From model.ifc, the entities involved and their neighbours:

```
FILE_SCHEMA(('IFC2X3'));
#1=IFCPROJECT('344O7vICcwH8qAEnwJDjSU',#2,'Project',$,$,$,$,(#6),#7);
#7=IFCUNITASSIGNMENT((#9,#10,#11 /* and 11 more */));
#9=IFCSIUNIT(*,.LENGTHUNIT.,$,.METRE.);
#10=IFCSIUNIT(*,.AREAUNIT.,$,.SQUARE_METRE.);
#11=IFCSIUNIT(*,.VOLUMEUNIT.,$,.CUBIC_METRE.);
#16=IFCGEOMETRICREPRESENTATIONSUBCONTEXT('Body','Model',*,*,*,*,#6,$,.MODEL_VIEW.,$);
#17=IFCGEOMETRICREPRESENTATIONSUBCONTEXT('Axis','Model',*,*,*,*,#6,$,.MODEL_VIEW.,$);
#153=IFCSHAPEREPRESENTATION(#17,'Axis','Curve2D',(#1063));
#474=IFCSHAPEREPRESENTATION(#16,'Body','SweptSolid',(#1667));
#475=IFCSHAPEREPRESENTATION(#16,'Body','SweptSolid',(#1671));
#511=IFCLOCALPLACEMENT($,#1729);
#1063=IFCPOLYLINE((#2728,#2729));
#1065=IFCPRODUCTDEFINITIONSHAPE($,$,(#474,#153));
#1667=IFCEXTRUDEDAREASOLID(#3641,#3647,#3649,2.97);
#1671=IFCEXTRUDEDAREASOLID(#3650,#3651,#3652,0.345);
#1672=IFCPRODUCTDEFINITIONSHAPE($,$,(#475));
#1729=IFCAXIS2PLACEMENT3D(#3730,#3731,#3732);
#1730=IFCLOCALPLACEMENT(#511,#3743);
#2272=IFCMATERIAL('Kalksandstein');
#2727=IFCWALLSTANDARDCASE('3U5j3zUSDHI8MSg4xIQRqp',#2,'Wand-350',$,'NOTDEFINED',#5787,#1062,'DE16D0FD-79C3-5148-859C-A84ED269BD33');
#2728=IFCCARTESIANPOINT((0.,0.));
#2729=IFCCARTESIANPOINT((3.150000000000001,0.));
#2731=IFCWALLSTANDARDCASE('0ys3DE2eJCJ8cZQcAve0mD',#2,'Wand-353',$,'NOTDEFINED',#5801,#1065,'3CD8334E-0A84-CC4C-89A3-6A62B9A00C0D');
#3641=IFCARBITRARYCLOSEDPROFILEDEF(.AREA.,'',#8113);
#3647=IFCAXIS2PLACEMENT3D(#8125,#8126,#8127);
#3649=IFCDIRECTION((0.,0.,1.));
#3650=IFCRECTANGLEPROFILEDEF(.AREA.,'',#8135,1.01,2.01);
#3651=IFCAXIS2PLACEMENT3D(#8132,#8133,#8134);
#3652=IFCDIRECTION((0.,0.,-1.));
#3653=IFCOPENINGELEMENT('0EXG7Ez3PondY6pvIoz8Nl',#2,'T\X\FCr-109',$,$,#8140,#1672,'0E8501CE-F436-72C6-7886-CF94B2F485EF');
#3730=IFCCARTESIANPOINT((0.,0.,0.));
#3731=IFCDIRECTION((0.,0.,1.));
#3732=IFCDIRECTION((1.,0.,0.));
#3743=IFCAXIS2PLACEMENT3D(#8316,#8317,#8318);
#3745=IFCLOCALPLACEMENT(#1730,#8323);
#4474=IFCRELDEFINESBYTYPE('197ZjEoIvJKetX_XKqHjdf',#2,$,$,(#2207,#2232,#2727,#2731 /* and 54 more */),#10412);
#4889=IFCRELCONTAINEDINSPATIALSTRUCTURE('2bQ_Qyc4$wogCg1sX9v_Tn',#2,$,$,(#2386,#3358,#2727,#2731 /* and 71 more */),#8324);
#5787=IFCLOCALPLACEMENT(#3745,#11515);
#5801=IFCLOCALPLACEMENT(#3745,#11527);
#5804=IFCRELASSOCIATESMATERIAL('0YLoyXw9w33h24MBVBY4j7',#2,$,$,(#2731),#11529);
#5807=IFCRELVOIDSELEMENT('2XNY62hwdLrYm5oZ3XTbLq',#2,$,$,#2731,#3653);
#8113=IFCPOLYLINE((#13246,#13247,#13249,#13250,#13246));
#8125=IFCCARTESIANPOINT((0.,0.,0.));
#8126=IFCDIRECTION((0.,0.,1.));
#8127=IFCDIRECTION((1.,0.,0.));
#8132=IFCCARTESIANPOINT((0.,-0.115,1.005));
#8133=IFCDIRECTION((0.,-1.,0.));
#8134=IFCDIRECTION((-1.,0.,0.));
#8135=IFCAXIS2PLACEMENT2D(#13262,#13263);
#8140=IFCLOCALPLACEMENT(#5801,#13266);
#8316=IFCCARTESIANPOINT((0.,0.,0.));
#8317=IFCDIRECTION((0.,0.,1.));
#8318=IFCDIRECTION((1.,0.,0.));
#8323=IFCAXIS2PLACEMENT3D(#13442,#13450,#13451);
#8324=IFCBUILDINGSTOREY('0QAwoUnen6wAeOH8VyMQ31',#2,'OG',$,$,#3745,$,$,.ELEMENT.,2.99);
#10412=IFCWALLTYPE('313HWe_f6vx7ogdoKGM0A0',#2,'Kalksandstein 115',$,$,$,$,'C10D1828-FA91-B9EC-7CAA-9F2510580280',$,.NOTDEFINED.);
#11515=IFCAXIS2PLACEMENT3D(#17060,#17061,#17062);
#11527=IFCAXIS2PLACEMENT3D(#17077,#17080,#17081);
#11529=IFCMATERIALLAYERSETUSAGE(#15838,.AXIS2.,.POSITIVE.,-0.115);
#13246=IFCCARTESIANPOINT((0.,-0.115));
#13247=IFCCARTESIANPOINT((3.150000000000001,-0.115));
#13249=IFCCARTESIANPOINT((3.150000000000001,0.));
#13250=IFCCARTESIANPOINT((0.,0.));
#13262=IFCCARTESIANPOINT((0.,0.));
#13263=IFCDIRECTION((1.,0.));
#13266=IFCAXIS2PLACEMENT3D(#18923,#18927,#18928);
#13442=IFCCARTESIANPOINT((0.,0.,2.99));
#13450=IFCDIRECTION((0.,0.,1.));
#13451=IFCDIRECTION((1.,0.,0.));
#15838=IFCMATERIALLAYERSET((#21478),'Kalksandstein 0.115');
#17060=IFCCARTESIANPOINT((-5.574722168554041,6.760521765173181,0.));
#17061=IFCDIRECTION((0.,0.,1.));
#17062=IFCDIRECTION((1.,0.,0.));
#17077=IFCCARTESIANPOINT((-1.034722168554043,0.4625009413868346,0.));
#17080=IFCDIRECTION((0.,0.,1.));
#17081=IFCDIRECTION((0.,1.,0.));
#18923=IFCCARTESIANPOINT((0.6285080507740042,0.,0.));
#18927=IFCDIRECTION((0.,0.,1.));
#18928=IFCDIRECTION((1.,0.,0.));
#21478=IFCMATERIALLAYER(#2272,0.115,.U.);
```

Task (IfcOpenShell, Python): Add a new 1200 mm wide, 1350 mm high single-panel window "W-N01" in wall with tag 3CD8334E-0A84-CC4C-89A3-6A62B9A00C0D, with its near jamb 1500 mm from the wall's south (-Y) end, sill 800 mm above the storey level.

```python
import numpy as np
import ifcopenshell
import ifcopenshell.api.feature
import ifcopenshell.api.geometry
import ifcopenshell.api.root
import ifcopenshell.api.spatial
import ifcopenshell.api.type
import ifcopenshell.geom
import ifcopenshell.util.element
import ifcopenshell.util.placement
import ifcopenshell.util.representation
import ifcopenshell.util.shape
import ifcopenshell.util.unit

model = ifcopenshell.open("model.ifc")
unit_scale = ifcopenshell.util.unit.calculate_unit_scale(model)
settings = ifcopenshell.geom.settings()


def volume(element):
    """Net volume in cubic metres, openings subtracted."""
    shape = ifcopenshell.geom.create_shape(settings, element)
    return ifcopenshell.util.shape.get_volume(shape.geometry)


wall = model.by_guid("0ys3DE2eJCJ8cZQcAve0mD")
storey = ifcopenshell.util.element.get_container(wall, ifc_class="IfcBuildingStorey")
context = ifcopenshell.util.representation.get_context(model, "Model", "Body", "MODEL_VIEW")
before = volume(wall)

width, height, from_end, sill = 1.2, 1.35, 1.5, 0.8  # metres

# The wall runs along its own X axis, and the end named is its -X end.
wall_shape = ifcopenshell.geom.create_shape(settings, wall)
x, y, z = ifcopenshell.util.shape.get_vertices(wall_shape.geometry).T
start = x.min() + from_end
face, thickness = float(y.min()), float(y.max() - y.min())
wall_matrix = ifcopenshell.util.placement.get_local_placement(wall.ObjectPlacement)
level = ifcopenshell.util.placement.get_local_placement(storey.ObjectPlacement)[2, 3]


def in_wall(x, y):
    """Placement at x, y metres in the wall's axes, at sill height."""
    matrix = wall_matrix.copy()
    matrix[:, 3] = wall_matrix @ np.array([x / unit_scale, y / unit_scale, 0.0, 1.0])
    matrix[2, 3] = level + sill / unit_scale
    return matrix


# Opening: a box that overshoots both wall faces by 50 mm.
opening = ifcopenshell.api.root.create_entity(model, ifc_class="IfcOpeningElement")
box = ifcopenshell.api.geometry.add_wall_representation(
    model, context=context, length=width, height=height, thickness=thickness + 0.1
)
ifcopenshell.api.geometry.assign_representation(model, product=opening, representation=box)
ifcopenshell.api.geometry.edit_object_placement(model, product=opening, matrix=in_wall(start, face - 0.05), is_si=False)
ifcopenshell.api.feature.add_feature(model, feature=opening, element=wall)

window = ifcopenshell.api.root.create_entity(model, ifc_class="IfcWindow", name="W-N01")
window.OverallWidth, window.OverallHeight = width / unit_scale, height / unit_scale
body = ifcopenshell.api.geometry.add_window_representation(
    model,
    context=context,
    overall_width=window.OverallWidth,
    overall_height=window.OverallHeight,
    partition_type="SINGLE_PANEL",
)
ifcopenshell.api.geometry.assign_representation(model, product=window, representation=body)
ifcopenshell.api.spatial.assign_container(model, products=[window], relating_structure=storey)
fills = ifcopenshell.api.feature.add_filling(model, opening=opening, element=window)
fills.OwnerHistory = window.OwnerHistory  # required in IFC2X3

# IFC2X3 keeps the operation on the window style.
style = ifcopenshell.api.root.create_entity(model, ifc_class="IfcWindowStyle", name="W-N01")
style.OperationType, style.ConstructionType = "SINGLE_PANEL", "NOTDEFINED"
style.ParameterTakesPrecedence = style.Sizeable = False
ifcopenshell.api.type.assign_type(model, related_objects=[window], relating_type=style)

# Centre the window in the wall's thickness.
ifcopenshell.api.geometry.edit_object_placement(model, product=window, matrix=in_wall(start, face), is_si=False)
window_shape = ifcopenshell.geom.create_shape(settings, window)
depth = ifcopenshell.util.shape.get_vertices(window_shape.geometry)[:, 1]
offset = face + thickness / 2 - (depth.min() + depth.max()) / 2
ifcopenshell.api.geometry.edit_object_placement(model, product=window, matrix=in_wall(start, offset), is_si=False)

after = volume(wall)

print(f"wall volume {before:.3f} -> {after:.3f} m3")

model.write("model_edited.ifc")
```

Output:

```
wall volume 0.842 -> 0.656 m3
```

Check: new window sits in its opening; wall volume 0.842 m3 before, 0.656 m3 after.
